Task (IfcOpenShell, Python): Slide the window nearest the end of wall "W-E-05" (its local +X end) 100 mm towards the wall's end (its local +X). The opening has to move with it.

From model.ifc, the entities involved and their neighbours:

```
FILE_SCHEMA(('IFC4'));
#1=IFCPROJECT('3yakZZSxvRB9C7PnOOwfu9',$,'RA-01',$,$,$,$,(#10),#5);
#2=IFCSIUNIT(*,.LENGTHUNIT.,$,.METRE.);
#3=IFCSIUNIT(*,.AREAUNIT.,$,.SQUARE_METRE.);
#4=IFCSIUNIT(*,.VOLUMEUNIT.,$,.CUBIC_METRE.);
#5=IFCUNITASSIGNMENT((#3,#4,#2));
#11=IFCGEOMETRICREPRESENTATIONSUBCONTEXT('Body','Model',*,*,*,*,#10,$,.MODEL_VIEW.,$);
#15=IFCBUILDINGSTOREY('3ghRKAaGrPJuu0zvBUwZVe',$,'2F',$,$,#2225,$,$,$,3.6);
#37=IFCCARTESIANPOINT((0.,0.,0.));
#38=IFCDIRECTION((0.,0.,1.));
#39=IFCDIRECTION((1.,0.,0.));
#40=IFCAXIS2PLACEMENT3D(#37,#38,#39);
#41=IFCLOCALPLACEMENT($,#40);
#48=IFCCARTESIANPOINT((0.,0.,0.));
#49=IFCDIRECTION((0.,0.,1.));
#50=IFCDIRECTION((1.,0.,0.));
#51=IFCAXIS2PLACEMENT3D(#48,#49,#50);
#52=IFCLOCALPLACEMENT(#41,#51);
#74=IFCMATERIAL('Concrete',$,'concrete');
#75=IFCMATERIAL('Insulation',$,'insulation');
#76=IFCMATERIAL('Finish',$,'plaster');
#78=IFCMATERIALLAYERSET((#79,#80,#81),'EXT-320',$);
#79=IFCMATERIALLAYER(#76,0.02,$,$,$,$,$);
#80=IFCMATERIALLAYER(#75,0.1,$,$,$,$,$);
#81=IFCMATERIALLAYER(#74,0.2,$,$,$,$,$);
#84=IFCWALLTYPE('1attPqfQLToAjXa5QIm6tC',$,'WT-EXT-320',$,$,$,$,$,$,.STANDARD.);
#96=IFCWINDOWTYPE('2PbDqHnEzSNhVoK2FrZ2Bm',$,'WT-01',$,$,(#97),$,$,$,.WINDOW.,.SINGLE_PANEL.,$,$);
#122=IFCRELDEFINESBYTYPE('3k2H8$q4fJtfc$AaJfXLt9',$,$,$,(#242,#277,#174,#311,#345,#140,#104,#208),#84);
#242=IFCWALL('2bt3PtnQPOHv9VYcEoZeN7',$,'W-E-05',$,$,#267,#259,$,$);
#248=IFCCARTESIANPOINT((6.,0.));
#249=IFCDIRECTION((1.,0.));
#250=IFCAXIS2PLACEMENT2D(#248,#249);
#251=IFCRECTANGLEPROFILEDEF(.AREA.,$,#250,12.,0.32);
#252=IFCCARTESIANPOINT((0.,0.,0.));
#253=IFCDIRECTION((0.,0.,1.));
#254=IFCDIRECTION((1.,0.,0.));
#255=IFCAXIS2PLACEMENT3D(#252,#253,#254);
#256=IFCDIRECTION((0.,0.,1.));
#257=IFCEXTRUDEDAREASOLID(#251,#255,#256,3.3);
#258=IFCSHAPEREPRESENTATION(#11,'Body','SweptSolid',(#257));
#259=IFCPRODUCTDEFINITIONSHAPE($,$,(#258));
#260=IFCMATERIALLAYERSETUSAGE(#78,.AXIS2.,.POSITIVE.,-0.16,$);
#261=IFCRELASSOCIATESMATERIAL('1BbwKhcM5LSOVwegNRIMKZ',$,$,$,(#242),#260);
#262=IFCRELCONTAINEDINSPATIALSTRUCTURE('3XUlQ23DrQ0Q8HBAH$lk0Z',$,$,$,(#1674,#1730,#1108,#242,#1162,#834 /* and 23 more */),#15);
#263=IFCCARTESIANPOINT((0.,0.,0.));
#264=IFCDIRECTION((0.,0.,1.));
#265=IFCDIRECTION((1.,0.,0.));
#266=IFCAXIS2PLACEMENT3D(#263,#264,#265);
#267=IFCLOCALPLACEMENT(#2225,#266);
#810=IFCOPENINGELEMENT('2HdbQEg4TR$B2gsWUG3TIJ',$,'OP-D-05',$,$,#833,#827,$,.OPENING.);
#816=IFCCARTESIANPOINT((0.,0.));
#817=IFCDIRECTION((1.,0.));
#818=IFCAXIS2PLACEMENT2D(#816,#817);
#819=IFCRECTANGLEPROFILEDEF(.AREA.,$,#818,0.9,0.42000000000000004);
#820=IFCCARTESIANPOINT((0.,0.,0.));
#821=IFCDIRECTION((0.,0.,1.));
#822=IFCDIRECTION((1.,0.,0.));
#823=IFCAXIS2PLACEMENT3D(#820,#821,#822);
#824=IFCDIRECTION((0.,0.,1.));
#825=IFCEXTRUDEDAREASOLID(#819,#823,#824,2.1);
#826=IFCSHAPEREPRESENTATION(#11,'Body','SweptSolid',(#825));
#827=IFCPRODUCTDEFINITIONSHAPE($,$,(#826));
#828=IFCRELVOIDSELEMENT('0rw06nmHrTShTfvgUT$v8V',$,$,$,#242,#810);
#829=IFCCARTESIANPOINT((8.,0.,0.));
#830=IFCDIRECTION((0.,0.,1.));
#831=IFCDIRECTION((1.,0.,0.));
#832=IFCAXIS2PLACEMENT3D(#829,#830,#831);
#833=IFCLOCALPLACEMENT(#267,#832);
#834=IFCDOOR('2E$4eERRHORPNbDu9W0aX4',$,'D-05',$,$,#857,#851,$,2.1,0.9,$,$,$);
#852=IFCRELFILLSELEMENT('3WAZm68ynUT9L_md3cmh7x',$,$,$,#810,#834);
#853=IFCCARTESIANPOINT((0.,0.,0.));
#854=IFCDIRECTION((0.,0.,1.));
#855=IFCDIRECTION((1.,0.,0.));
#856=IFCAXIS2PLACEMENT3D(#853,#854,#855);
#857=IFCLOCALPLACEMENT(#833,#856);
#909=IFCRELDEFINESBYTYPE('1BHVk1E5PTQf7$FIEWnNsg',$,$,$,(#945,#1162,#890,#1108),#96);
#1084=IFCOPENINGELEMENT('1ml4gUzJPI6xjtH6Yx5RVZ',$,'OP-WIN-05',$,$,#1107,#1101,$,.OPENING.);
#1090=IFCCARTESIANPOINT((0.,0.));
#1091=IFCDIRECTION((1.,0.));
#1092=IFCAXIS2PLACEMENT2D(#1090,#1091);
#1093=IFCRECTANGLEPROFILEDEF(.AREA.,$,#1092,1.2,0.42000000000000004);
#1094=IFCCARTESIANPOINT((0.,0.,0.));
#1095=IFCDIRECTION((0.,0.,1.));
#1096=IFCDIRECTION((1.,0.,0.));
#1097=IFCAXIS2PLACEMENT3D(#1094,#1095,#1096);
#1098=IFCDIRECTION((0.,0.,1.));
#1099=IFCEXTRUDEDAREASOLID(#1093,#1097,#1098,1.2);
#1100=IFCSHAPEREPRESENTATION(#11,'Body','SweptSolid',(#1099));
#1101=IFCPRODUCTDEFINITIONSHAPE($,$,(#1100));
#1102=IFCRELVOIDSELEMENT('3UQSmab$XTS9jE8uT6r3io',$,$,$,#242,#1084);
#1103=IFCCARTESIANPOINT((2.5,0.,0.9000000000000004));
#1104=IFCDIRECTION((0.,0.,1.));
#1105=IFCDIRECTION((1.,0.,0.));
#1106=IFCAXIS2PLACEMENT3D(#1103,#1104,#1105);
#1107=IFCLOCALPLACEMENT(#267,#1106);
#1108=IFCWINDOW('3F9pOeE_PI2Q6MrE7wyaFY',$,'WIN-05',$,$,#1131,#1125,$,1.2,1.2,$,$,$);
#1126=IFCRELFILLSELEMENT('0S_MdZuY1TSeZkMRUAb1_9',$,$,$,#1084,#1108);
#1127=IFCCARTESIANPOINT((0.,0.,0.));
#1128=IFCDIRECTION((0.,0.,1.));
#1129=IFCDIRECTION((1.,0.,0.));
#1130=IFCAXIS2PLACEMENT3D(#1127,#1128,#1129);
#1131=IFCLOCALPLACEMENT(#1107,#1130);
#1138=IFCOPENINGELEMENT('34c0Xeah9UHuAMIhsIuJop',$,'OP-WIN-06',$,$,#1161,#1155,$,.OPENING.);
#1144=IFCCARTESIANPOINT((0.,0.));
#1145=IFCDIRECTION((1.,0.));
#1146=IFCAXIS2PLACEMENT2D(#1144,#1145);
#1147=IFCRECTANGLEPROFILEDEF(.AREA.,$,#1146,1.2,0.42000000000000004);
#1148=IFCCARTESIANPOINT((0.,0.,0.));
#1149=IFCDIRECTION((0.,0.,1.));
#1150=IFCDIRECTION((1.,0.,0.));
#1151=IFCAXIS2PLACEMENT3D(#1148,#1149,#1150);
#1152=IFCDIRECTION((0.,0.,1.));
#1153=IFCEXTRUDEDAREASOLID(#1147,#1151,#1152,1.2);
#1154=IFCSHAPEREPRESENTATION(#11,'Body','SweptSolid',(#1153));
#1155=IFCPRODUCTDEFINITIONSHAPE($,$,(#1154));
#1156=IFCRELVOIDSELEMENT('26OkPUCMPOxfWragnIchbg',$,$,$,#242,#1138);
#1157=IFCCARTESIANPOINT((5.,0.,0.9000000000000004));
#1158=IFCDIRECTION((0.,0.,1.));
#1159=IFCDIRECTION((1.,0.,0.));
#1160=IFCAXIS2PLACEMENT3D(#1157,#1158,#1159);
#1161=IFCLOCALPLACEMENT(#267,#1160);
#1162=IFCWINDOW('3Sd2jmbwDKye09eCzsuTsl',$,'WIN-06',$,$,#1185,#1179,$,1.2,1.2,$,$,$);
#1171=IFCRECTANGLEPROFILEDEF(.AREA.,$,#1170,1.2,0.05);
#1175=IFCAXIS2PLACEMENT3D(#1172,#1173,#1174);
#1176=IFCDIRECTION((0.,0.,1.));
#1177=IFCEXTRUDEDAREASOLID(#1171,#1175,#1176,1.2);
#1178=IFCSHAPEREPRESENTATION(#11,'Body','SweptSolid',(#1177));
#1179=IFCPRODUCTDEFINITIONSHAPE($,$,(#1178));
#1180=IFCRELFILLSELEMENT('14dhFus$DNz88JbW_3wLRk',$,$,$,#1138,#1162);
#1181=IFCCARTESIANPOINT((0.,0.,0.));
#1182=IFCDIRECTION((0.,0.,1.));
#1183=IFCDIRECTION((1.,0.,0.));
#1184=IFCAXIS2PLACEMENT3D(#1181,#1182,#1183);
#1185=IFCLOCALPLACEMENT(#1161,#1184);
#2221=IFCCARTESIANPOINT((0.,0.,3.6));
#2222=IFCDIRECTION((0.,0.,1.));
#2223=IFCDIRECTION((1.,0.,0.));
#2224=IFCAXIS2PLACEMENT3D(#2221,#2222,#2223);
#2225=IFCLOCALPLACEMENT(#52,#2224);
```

```python
import ifcopenshell
import ifcopenshell.api.geometry
import ifcopenshell.util.placement
import ifcopenshell.util.unit

model = ifcopenshell.open("model.ifc")
unit_scale = ifcopenshell.util.unit.calculate_unit_scale(model)

window = model.by_guid("3Sd2jmbwDKye09eCzsuTsl")
opening = window.FillsVoids[0].RelatingOpeningElement
wall = opening.VoidsElements[0].RelatingBuildingElement

wall_matrix = ifcopenshell.util.placement.get_local_placement(wall.ObjectPlacement)
shift = wall_matrix[:3, 0] * 0.1 / unit_scale
before = ifcopenshell.util.placement.get_local_placement(window.ObjectPlacement)[:3, 3].copy()

# The window is placed relative to its opening, so it follows when the opening moves.
matrix = ifcopenshell.util.placement.get_local_placement(opening.ObjectPlacement)
matrix[:3, 3] += shift
ifcopenshell.api.geometry.edit_object_placement(
    model, product=opening, matrix=matrix, is_si=False, should_transform_children=True
)

after = ifcopenshell.util.placement.get_local_placement(window.ObjectPlacement)[:3, 3]
print("window moved by", (after - before).round(3) + 0.0)

model.write("model-out.ifc")
```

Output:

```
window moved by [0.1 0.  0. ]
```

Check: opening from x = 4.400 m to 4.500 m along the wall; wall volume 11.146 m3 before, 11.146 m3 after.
